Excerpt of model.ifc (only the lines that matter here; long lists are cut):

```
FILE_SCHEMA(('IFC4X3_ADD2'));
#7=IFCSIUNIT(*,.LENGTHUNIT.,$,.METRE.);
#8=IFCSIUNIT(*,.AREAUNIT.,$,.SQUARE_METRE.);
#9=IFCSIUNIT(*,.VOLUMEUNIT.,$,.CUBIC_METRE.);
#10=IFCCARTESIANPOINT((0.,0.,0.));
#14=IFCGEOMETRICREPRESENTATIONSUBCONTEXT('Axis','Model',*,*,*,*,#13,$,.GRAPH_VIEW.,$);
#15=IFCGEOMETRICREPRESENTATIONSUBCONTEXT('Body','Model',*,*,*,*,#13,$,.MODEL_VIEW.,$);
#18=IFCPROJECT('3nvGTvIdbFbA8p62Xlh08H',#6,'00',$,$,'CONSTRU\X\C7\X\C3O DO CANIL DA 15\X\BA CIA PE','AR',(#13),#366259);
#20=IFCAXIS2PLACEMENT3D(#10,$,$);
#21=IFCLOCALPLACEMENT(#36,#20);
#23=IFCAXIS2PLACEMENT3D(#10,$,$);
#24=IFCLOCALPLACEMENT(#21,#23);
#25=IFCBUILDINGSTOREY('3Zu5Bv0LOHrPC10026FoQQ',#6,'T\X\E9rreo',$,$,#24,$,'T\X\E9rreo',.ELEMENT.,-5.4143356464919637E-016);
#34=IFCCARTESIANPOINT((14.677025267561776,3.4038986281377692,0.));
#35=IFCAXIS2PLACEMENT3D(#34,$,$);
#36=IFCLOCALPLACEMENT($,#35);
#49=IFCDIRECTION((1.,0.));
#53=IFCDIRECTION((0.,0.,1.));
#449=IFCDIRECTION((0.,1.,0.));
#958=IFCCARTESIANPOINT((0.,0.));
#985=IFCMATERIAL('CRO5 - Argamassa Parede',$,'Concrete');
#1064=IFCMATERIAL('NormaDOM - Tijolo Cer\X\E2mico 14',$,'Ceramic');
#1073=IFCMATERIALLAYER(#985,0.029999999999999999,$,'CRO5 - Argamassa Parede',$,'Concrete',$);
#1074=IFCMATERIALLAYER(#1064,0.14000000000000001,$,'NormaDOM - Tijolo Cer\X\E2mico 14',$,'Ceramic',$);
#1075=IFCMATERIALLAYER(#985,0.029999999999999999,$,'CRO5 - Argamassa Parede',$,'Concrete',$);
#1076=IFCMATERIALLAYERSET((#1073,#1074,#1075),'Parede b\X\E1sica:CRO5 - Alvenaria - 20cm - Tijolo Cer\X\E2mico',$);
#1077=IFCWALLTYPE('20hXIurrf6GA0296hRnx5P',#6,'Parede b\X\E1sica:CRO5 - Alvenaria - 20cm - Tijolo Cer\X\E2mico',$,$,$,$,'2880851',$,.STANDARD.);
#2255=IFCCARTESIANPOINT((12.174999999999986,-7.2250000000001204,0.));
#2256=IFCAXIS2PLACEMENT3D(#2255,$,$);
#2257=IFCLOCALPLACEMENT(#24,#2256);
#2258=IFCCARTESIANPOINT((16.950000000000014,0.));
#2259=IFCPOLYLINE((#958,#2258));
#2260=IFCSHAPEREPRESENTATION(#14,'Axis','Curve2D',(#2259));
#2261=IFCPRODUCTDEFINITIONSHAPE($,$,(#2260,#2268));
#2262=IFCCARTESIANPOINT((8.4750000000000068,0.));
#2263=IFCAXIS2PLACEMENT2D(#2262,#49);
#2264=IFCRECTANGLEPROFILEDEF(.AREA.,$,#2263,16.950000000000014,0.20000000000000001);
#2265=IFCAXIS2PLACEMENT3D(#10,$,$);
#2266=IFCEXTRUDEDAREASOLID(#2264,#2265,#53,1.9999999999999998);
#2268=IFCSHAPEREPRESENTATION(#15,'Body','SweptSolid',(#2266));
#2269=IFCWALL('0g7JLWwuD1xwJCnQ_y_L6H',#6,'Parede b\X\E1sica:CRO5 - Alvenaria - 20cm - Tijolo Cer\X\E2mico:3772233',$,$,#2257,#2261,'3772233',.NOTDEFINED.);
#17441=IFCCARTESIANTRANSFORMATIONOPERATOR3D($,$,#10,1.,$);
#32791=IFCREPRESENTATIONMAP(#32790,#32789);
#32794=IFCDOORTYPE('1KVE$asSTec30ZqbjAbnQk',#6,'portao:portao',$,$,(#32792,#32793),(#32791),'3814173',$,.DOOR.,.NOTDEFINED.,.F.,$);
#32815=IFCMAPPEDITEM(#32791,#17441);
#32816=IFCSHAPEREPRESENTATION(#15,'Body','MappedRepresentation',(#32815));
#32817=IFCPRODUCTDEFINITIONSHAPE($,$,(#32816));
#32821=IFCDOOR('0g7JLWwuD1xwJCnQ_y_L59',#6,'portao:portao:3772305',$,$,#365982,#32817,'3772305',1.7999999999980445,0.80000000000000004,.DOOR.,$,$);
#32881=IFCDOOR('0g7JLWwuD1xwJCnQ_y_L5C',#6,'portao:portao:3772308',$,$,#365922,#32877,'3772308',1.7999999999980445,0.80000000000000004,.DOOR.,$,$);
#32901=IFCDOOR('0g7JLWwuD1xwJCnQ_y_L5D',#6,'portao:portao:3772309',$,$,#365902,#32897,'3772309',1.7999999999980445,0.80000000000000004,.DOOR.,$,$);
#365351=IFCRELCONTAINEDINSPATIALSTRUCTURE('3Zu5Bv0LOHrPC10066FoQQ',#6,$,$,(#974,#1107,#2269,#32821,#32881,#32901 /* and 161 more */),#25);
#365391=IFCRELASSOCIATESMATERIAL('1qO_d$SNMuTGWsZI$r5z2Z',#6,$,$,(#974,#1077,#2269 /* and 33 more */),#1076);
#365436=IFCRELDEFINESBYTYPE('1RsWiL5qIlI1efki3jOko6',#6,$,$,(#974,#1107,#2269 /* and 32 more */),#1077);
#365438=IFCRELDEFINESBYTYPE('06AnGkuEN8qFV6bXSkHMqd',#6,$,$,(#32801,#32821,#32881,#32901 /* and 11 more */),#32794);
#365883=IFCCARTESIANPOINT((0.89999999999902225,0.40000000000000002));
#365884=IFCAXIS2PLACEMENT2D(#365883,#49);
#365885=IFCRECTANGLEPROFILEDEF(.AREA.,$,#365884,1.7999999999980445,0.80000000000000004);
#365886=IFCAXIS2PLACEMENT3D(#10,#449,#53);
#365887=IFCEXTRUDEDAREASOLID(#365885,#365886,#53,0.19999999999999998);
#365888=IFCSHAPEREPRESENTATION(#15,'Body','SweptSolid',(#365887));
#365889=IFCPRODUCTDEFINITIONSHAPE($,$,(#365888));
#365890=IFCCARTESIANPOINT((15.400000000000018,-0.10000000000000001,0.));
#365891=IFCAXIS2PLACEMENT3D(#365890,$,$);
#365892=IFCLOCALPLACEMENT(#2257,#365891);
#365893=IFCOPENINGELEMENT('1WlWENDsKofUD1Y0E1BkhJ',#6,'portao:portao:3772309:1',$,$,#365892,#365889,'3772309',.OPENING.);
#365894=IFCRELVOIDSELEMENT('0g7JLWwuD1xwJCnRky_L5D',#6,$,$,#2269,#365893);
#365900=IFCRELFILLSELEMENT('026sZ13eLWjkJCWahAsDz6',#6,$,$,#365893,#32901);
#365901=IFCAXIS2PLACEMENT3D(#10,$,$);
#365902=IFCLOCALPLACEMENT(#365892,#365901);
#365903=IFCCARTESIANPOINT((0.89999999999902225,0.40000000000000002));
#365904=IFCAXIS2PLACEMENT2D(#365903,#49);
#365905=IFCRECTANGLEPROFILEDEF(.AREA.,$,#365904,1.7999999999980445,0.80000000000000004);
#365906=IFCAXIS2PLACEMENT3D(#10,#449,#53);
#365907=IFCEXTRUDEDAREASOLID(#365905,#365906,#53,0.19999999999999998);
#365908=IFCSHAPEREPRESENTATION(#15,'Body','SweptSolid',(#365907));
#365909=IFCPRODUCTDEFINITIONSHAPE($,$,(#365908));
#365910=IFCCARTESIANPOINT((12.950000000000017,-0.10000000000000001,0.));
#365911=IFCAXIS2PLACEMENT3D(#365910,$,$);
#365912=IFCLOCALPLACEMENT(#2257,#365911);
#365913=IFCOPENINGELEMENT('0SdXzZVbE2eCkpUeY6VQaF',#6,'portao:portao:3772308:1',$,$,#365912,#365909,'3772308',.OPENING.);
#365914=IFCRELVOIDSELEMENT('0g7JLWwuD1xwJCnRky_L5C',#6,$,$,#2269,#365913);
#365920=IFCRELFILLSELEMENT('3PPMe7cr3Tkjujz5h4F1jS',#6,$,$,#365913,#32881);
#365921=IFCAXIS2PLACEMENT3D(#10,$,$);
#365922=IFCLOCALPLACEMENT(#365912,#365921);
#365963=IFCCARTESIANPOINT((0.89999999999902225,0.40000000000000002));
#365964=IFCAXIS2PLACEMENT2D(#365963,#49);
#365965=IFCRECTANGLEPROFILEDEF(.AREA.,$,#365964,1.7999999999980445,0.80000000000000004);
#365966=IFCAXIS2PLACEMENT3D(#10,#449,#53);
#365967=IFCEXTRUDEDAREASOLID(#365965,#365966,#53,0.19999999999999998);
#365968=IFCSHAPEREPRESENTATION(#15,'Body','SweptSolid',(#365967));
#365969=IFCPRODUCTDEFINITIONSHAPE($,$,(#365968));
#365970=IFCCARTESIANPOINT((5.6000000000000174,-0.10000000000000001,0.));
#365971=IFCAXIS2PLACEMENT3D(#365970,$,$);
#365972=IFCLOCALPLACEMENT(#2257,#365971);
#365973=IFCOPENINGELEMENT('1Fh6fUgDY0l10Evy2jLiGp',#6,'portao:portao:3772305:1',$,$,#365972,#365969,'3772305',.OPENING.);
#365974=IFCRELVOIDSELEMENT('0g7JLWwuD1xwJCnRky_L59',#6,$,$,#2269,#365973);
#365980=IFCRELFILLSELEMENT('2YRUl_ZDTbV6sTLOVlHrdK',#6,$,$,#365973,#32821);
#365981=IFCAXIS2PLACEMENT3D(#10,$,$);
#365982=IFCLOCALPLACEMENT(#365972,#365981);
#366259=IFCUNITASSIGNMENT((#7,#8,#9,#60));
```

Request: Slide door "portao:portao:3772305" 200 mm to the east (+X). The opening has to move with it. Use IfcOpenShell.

```python
import ifcopenshell
import ifcopenshell.api.geometry
import ifcopenshell.util.placement
import ifcopenshell.util.unit

model = ifcopenshell.open("model.ifc")
unit_scale = ifcopenshell.util.unit.calculate_unit_scale(model)

door = model.by_guid("0g7JLWwuD1xwJCnQ_y_L59")
opening = door.FillsVoids[0].RelatingOpeningElement
wall = opening.VoidsElements[0].RelatingBuildingElement

wall_matrix = ifcopenshell.util.placement.get_local_placement(wall.ObjectPlacement)
shift = wall_matrix[:3, 0] * 0.2 / unit_scale
before = ifcopenshell.util.placement.get_local_placement(door.ObjectPlacement)[:3, 3].copy()

# The door is placed relative to its opening, so it follows when the opening moves.
matrix = ifcopenshell.util.placement.get_local_placement(opening.ObjectPlacement)
matrix[:3, 3] += shift
ifcopenshell.api.geometry.edit_object_placement(
    model, product=opening, matrix=matrix, is_si=False, should_transform_children=True
)

after = ifcopenshell.util.placement.get_local_placement(door.ObjectPlacement)[:3, 3]
print("door moved by", (after - before).round(3) + 0.0)

model.write("model_rev.ifc")
```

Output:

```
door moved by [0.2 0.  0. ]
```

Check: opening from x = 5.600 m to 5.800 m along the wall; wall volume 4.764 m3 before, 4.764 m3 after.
